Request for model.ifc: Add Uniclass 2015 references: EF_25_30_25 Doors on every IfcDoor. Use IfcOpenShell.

First a look at what the model holds.

```python
import ifcopenshell

model = ifcopenshell.open("model.ifc")
print(model.schema)
print("classifications:", [c.Name for c in model.by_type("IfcClassification")])
for ifc_class in ("IfcDoor", "IfcRoof", "IfcStair", "IfcWall", "IfcWindow"):
    print(ifc_class, len(model.by_type(ifc_class)))
```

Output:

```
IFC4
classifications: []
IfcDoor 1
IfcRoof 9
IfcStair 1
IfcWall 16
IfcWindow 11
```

```python
import ifcopenshell
import ifcopenshell.api.classification

model = ifcopenshell.open("model.ifc")

system = ifcopenshell.api.classification.add_classification(model, classification="Uniclass 2015")

codes = {
    "IfcDoor": ("EF_25_30_25", "Doors"),
}
for ifc_class, (code, name) in codes.items():
    products = model.by_type(ifc_class)
    ifcopenshell.api.classification.add_reference(
        model, products=products, classification=system, identification=code, name=name
    )
    print(code, len(products))

model.write("model_edited.ifc")
```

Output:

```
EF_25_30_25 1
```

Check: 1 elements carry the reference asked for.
